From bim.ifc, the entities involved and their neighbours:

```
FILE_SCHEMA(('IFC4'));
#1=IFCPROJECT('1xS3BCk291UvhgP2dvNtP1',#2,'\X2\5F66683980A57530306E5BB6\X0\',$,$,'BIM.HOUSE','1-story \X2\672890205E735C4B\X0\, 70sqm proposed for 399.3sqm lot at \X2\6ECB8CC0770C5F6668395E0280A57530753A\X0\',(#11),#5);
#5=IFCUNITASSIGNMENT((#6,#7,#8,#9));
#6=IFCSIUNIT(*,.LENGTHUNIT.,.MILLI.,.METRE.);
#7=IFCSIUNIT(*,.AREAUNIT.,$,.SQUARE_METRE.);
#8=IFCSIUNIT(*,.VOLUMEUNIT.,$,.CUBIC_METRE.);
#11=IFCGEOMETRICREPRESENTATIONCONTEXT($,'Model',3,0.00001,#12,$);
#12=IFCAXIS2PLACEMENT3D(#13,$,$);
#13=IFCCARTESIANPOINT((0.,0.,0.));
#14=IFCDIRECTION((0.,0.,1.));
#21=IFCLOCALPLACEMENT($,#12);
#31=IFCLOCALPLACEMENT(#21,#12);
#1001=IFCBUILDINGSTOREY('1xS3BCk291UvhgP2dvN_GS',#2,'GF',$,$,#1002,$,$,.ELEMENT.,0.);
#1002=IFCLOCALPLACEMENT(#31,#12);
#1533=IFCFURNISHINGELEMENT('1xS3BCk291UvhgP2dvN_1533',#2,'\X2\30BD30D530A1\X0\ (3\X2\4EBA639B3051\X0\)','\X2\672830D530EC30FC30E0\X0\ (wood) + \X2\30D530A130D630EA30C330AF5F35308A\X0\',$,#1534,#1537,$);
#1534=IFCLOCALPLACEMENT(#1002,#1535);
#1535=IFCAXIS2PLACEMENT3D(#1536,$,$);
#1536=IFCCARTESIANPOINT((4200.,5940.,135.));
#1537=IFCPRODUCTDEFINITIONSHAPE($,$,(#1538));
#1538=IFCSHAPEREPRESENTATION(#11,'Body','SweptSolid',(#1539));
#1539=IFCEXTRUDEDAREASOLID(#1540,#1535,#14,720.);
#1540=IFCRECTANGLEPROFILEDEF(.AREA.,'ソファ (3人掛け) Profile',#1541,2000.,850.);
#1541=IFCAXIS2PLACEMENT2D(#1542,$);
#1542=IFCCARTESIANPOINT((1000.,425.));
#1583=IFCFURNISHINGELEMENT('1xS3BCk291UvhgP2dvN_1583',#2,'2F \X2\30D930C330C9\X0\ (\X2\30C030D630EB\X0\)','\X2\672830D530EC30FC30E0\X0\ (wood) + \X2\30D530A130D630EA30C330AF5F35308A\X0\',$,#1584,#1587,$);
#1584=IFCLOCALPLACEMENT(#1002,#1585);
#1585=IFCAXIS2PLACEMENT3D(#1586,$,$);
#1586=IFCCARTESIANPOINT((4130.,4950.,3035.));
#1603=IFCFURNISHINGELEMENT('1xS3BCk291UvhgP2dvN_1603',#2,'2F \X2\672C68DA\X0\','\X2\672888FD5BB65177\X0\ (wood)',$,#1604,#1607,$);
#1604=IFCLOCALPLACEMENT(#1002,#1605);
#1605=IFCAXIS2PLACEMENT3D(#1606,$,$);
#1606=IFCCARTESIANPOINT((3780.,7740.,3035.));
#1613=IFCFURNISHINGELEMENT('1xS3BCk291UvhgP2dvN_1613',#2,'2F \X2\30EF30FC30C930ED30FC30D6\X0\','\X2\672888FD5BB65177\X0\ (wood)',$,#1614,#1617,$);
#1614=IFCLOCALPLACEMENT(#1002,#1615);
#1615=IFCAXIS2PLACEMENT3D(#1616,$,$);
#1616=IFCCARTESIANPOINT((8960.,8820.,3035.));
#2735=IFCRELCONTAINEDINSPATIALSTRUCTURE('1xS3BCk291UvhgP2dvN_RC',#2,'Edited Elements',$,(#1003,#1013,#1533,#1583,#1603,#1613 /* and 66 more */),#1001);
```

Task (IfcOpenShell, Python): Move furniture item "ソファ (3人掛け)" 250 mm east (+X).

```python
import ifcopenshell
import ifcopenshell.api.geometry
import ifcopenshell.util.placement
import ifcopenshell.util.unit

model = ifcopenshell.open("bim.ifc")
unit_scale = ifcopenshell.util.unit.calculate_unit_scale(model)

item = model.by_id(1533)
matrix = ifcopenshell.util.placement.get_local_placement(item.ObjectPlacement)
matrix[0, 3] += 0.25 / unit_scale
ifcopenshell.api.geometry.edit_object_placement(model, product=item, matrix=matrix, is_si=False)

print(ifcopenshell.util.placement.get_local_placement(item.ObjectPlacement).round(3) + 0.0)

model.write("bim_v2.ifc")
```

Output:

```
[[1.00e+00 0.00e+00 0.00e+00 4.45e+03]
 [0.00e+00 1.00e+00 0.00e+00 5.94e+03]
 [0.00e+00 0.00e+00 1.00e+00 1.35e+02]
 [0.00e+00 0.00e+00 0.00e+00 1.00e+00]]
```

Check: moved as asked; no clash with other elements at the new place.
